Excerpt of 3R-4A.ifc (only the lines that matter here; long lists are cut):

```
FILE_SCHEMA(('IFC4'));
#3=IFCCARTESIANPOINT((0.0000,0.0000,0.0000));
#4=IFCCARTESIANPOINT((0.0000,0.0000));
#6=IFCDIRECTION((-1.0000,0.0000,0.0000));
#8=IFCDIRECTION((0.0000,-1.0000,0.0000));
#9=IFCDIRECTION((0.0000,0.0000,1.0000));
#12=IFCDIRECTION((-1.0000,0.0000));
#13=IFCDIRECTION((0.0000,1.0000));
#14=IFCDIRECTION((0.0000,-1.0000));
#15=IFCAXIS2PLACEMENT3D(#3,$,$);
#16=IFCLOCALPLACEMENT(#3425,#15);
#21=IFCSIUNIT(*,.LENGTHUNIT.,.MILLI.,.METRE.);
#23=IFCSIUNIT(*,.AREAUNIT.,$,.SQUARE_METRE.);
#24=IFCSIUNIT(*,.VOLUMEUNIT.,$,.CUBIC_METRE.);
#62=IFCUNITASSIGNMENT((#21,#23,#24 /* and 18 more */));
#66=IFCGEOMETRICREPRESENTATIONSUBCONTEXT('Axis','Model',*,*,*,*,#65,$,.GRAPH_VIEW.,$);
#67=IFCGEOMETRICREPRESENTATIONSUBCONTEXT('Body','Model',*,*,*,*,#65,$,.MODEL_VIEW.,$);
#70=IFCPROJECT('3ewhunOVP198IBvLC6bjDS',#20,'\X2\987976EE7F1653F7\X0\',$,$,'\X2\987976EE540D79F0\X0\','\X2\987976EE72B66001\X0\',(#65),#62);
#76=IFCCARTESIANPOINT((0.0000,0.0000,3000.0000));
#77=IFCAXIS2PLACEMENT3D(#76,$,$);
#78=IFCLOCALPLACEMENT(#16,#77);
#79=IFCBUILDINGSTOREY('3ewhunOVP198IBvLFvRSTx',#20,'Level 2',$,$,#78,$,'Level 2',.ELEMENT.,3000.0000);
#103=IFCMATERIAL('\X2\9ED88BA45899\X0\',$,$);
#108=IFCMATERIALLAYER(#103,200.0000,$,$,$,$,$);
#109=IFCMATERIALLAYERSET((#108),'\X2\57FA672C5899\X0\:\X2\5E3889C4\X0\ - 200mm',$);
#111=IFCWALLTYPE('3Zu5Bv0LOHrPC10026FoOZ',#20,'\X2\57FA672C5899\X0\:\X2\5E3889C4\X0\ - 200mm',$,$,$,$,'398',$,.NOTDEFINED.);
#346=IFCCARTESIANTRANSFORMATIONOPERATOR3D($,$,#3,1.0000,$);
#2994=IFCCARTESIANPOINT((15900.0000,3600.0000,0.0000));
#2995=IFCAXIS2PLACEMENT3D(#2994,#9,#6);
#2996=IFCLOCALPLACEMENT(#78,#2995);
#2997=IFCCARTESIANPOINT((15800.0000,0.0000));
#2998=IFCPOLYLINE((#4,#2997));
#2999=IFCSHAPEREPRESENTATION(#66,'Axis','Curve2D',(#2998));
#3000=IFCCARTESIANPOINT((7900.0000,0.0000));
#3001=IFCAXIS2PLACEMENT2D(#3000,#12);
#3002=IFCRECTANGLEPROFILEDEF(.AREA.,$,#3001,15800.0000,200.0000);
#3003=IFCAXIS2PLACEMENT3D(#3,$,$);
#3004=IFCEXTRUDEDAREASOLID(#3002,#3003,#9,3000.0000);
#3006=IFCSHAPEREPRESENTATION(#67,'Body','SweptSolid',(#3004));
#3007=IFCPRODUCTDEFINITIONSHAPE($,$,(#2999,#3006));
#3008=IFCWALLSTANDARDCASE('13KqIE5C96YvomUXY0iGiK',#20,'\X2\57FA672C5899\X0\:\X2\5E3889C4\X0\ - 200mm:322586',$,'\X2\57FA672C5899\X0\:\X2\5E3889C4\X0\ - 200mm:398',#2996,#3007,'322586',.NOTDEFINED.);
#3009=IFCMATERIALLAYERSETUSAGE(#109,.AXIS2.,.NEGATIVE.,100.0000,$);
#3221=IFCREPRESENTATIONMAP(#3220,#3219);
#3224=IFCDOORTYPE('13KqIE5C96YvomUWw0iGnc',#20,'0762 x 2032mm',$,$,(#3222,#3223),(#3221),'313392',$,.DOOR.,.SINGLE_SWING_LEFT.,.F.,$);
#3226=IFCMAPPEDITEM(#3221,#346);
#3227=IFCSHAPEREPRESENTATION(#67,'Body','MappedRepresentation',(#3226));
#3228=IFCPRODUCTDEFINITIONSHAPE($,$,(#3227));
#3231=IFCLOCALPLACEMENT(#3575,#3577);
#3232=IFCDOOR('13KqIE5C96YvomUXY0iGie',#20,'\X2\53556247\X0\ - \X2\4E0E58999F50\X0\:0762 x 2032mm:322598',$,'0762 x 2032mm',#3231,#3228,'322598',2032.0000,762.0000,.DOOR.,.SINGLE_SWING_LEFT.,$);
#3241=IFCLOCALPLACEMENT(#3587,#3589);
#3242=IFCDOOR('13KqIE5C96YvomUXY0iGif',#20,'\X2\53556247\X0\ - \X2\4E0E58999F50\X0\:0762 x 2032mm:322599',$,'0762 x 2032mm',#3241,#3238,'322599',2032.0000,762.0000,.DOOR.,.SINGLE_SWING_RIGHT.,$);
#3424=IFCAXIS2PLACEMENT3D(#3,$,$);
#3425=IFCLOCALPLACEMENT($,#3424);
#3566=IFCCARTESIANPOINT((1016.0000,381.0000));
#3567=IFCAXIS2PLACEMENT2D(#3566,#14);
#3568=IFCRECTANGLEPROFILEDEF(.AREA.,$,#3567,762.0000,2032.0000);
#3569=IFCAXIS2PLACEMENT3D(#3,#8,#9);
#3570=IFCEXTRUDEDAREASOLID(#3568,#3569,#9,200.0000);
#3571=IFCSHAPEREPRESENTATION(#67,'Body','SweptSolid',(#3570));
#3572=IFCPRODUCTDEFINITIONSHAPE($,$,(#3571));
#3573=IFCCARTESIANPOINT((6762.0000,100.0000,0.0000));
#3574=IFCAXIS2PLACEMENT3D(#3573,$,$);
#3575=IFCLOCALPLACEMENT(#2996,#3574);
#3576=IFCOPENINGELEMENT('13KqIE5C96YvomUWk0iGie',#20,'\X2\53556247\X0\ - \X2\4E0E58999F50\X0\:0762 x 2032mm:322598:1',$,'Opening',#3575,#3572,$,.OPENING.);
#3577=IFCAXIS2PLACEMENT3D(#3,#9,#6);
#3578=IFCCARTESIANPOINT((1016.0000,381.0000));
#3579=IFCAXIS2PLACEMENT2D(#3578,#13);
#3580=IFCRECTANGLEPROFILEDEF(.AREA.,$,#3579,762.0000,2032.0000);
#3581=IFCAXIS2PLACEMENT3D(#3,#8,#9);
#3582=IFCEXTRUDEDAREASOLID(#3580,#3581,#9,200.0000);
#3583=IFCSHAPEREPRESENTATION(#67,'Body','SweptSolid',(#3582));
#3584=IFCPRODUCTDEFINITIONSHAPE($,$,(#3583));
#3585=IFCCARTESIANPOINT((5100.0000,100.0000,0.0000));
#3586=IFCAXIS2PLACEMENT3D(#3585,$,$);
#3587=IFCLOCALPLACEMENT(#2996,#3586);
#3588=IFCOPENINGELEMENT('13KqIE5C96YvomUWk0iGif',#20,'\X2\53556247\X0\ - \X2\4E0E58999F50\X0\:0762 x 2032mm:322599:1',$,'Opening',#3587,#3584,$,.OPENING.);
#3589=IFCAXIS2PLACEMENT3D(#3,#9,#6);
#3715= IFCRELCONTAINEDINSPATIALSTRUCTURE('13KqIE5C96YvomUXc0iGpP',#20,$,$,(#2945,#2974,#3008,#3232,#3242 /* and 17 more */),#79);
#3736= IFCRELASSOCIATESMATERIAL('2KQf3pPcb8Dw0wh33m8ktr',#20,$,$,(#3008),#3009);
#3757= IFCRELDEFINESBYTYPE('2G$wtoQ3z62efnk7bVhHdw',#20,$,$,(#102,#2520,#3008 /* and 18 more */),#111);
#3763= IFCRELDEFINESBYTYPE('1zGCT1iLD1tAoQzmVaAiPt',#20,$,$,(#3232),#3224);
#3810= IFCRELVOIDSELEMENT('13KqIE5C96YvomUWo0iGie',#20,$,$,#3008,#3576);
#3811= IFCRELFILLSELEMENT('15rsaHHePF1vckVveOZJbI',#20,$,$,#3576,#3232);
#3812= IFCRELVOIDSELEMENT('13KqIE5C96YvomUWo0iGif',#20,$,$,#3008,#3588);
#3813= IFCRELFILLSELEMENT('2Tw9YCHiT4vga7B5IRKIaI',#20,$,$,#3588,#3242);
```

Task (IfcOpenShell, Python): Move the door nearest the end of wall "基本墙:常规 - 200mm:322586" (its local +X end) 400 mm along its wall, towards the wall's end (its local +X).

```python
import ifcopenshell
import ifcopenshell.api.geometry
import ifcopenshell.util.placement
import ifcopenshell.util.unit

model = ifcopenshell.open("3R-4A.ifc")
unit_scale = ifcopenshell.util.unit.calculate_unit_scale(model)

door = model.by_guid("13KqIE5C96YvomUXY0iGie")
opening = door.FillsVoids[0].RelatingOpeningElement
wall = opening.VoidsElements[0].RelatingBuildingElement

wall_matrix = ifcopenshell.util.placement.get_local_placement(wall.ObjectPlacement)
shift = wall_matrix[:3, 0] * 0.4 / unit_scale
before = ifcopenshell.util.placement.get_local_placement(door.ObjectPlacement)[:3, 3].copy()

# The door is placed relative to its opening, so it follows when the opening moves.
matrix = ifcopenshell.util.placement.get_local_placement(opening.ObjectPlacement)
matrix[:3, 3] += shift
ifcopenshell.api.geometry.edit_object_placement(
    model, product=opening, matrix=matrix, is_si=False, should_transform_children=True
)

after = ifcopenshell.util.placement.get_local_placement(door.ObjectPlacement)[:3, 3]
print("door moved by", (after - before).round(3) + 0.0)

model.write("3R-4A-out.ifc")
```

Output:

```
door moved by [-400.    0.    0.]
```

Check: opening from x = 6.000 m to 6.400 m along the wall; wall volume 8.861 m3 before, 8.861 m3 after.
